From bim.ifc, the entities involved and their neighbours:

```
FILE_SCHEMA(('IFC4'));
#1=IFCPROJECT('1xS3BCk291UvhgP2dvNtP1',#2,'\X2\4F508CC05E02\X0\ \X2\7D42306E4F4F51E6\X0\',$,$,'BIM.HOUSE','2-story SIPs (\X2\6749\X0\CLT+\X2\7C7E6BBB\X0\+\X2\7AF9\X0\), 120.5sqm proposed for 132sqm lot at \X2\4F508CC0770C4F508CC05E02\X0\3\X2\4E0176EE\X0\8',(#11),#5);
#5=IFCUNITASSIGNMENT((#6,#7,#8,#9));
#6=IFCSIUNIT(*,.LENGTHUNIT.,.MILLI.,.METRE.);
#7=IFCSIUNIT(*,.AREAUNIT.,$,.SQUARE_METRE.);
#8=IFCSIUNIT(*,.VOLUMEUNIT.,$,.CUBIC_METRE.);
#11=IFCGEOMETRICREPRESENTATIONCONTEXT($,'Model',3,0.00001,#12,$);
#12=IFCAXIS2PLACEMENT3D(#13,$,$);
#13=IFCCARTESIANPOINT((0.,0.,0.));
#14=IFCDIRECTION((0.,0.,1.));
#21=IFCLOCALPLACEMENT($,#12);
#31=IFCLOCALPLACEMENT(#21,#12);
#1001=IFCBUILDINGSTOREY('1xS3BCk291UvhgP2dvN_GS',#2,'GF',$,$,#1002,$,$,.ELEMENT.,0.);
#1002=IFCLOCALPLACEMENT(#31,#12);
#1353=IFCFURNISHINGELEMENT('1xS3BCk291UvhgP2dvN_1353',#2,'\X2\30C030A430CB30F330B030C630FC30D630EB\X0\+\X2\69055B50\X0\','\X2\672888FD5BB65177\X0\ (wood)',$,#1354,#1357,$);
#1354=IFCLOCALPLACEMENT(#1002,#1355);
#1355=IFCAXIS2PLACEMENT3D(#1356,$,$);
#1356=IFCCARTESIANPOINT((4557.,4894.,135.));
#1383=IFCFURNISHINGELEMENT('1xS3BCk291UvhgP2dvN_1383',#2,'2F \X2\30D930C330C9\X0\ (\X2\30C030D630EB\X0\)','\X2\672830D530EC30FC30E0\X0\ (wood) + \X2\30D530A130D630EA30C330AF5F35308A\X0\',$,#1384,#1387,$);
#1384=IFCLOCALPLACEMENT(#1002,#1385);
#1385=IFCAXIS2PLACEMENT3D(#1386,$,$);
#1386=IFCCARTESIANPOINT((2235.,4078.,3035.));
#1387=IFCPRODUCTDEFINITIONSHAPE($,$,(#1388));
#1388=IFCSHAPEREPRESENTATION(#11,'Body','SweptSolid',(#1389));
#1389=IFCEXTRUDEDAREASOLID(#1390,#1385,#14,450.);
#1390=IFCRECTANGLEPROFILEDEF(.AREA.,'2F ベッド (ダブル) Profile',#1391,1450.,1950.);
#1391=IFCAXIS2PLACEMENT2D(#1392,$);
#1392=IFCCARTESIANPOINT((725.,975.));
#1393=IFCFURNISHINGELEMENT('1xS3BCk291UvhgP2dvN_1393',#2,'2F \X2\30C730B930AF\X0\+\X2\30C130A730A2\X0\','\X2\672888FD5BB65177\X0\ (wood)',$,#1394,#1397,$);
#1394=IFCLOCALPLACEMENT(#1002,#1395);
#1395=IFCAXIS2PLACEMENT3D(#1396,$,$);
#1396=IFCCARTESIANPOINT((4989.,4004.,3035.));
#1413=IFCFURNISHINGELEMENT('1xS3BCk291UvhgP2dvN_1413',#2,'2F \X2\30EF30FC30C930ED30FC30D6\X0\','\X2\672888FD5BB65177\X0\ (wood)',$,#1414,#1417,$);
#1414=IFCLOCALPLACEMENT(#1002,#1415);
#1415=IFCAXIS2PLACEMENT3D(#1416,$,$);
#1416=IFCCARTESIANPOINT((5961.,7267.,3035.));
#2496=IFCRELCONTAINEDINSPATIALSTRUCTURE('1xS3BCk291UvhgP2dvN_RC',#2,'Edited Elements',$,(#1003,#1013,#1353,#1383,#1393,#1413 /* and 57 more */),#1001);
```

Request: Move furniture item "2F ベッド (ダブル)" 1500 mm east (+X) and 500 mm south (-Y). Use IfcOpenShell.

```python
import ifcopenshell
import ifcopenshell.api.geometry
import ifcopenshell.util.placement
import ifcopenshell.util.unit

model = ifcopenshell.open("bim.ifc")
unit_scale = ifcopenshell.util.unit.calculate_unit_scale(model)

item = model.by_guid("1xS3BCk291UvhgP2dvN_1383")
matrix = ifcopenshell.util.placement.get_local_placement(item.ObjectPlacement)
matrix[0, 3] += 1.5 / unit_scale
matrix[1, 3] -= 0.5 / unit_scale
ifcopenshell.api.geometry.edit_object_placement(model, product=item, matrix=matrix, is_si=False)

print(ifcopenshell.util.placement.get_local_placement(item.ObjectPlacement).round(3) + 0.0)

model.write("bim_updated.ifc")
```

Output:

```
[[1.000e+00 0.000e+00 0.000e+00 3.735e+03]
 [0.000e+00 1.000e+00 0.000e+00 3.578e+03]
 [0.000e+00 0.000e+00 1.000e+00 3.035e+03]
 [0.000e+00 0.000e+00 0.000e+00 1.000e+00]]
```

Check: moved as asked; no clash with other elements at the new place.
